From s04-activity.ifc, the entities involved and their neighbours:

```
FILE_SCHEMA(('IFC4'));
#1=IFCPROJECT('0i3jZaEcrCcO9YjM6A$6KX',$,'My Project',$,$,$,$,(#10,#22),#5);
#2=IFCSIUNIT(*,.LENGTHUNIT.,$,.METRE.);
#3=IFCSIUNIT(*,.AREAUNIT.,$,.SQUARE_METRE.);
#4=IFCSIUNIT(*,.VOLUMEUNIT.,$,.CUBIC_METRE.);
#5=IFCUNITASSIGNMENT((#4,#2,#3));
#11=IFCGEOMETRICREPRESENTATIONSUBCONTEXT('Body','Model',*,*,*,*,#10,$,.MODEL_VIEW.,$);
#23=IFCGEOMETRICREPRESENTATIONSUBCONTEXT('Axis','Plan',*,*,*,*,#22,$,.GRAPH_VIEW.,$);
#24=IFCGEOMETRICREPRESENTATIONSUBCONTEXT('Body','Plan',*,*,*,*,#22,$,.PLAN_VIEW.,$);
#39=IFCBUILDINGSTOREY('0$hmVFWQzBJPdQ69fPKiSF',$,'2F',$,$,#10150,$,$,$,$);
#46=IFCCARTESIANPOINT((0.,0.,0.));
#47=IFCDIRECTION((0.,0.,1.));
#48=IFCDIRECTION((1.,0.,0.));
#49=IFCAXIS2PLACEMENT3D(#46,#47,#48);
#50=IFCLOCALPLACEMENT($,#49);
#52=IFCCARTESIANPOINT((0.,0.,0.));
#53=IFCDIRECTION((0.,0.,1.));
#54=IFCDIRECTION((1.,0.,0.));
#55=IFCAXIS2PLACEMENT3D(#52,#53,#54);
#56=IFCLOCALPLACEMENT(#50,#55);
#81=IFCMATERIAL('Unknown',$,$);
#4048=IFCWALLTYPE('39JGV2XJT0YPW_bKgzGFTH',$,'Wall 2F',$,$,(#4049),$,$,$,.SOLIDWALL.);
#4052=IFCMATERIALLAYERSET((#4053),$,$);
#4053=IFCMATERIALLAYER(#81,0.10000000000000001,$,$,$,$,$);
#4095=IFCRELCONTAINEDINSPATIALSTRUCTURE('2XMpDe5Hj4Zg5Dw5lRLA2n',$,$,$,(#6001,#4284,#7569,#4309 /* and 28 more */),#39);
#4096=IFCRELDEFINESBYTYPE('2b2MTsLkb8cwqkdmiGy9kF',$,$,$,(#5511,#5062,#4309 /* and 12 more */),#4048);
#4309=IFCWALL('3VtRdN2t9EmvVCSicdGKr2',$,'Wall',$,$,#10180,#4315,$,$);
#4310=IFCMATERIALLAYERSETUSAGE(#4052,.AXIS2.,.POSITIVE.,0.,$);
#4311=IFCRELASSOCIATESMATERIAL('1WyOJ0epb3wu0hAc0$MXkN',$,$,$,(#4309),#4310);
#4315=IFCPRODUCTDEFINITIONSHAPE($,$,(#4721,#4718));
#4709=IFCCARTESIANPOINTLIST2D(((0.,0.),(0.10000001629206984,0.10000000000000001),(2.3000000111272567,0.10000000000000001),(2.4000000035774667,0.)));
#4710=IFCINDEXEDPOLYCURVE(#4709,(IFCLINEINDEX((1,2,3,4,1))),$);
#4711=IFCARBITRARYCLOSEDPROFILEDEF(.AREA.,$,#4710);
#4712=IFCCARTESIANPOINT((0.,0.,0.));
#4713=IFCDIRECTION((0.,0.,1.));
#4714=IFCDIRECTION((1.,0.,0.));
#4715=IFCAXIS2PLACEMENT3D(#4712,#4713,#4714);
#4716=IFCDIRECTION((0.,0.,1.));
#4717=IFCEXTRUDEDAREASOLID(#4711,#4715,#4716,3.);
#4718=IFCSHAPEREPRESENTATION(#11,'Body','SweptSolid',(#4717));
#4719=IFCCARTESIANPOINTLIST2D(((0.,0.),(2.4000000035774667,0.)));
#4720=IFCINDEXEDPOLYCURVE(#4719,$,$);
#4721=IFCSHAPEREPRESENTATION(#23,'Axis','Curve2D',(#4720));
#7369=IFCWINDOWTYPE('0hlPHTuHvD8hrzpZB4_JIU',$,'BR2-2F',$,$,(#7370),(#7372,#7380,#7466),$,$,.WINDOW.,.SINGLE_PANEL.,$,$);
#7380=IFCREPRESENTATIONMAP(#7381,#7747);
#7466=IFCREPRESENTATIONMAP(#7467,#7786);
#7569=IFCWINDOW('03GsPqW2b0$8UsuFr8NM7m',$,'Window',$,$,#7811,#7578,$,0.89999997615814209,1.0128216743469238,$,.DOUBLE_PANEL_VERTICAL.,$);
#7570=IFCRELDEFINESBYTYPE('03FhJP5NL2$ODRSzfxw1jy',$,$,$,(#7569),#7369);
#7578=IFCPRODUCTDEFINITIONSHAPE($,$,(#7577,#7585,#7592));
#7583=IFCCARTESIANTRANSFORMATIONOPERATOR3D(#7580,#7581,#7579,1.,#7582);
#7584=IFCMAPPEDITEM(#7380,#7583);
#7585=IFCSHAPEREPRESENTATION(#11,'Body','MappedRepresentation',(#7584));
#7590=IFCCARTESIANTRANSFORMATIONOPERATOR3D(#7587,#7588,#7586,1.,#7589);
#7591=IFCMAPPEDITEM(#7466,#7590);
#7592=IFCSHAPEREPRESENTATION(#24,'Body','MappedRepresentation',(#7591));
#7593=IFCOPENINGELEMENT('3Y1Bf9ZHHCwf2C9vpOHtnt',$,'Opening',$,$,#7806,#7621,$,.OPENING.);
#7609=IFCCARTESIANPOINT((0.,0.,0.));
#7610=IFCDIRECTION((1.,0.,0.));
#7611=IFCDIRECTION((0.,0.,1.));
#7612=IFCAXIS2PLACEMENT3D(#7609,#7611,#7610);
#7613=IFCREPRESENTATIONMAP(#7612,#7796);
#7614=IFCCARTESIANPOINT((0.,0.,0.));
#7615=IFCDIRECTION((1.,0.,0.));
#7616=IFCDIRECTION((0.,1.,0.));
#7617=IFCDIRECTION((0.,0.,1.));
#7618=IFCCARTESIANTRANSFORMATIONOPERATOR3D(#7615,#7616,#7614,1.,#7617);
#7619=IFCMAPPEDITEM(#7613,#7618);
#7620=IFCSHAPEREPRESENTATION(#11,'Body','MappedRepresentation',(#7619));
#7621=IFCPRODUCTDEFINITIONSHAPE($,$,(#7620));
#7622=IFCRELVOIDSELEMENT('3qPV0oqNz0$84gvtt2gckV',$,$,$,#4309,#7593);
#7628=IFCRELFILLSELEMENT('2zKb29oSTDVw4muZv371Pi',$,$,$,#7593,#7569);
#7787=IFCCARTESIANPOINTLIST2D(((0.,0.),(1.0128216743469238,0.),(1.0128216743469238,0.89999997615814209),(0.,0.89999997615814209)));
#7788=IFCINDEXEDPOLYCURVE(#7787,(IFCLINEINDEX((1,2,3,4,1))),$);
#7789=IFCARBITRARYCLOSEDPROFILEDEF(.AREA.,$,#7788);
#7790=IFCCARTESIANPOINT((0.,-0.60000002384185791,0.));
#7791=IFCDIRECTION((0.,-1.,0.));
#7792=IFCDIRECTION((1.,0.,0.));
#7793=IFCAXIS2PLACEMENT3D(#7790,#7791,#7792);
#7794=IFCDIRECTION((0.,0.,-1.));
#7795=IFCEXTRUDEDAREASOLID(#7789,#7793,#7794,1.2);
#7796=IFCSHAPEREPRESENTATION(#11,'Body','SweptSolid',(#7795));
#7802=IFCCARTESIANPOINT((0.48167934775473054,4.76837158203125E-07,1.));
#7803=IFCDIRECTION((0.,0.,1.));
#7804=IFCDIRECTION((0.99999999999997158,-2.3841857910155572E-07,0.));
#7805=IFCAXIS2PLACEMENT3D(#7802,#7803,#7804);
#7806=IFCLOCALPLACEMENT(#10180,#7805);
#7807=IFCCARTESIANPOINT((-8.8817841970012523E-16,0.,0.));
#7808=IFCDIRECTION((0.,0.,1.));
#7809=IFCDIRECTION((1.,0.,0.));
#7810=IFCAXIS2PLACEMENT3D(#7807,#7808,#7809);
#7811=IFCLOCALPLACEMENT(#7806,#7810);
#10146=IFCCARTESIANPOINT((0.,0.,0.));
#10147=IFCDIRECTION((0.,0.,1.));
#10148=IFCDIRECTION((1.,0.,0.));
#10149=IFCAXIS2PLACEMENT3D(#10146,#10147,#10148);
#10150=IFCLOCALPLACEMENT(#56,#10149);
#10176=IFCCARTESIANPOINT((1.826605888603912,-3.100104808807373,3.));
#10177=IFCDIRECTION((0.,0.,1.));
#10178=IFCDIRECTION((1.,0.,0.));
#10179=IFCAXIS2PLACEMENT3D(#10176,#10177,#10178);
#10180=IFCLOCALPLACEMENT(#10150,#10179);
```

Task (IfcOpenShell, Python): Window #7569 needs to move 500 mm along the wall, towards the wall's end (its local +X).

```python
import ifcopenshell
import ifcopenshell.api.geometry
import ifcopenshell.util.placement

model = ifcopenshell.open("s04-activity.ifc")

window = model.by_guid("03GsPqW2b0$8UsuFr8NM7m")
opening = window.FillsVoids[0].RelatingOpeningElement
wall = opening.VoidsElements[0].RelatingBuildingElement

wall_matrix = ifcopenshell.util.placement.get_local_placement(wall.ObjectPlacement)
shift = wall_matrix[:3, 0] * 0.5
before = ifcopenshell.util.placement.get_local_placement(window.ObjectPlacement)[:3, 3].copy()

# The window is placed relative to its opening, so it follows when the opening moves.
matrix = ifcopenshell.util.placement.get_local_placement(opening.ObjectPlacement)
matrix[:3, 3] += shift
ifcopenshell.api.geometry.edit_object_placement(
    model, product=opening, matrix=matrix, is_si=False, should_transform_children=True
)

after = ifcopenshell.util.placement.get_local_placement(window.ObjectPlacement)[:3, 3]
print("window moved by", (after - before).round(3) + 0.0)

model.write("s04-activity_updated.ifc")
```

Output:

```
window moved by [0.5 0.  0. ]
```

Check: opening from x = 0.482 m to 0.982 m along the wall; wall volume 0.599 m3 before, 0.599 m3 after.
